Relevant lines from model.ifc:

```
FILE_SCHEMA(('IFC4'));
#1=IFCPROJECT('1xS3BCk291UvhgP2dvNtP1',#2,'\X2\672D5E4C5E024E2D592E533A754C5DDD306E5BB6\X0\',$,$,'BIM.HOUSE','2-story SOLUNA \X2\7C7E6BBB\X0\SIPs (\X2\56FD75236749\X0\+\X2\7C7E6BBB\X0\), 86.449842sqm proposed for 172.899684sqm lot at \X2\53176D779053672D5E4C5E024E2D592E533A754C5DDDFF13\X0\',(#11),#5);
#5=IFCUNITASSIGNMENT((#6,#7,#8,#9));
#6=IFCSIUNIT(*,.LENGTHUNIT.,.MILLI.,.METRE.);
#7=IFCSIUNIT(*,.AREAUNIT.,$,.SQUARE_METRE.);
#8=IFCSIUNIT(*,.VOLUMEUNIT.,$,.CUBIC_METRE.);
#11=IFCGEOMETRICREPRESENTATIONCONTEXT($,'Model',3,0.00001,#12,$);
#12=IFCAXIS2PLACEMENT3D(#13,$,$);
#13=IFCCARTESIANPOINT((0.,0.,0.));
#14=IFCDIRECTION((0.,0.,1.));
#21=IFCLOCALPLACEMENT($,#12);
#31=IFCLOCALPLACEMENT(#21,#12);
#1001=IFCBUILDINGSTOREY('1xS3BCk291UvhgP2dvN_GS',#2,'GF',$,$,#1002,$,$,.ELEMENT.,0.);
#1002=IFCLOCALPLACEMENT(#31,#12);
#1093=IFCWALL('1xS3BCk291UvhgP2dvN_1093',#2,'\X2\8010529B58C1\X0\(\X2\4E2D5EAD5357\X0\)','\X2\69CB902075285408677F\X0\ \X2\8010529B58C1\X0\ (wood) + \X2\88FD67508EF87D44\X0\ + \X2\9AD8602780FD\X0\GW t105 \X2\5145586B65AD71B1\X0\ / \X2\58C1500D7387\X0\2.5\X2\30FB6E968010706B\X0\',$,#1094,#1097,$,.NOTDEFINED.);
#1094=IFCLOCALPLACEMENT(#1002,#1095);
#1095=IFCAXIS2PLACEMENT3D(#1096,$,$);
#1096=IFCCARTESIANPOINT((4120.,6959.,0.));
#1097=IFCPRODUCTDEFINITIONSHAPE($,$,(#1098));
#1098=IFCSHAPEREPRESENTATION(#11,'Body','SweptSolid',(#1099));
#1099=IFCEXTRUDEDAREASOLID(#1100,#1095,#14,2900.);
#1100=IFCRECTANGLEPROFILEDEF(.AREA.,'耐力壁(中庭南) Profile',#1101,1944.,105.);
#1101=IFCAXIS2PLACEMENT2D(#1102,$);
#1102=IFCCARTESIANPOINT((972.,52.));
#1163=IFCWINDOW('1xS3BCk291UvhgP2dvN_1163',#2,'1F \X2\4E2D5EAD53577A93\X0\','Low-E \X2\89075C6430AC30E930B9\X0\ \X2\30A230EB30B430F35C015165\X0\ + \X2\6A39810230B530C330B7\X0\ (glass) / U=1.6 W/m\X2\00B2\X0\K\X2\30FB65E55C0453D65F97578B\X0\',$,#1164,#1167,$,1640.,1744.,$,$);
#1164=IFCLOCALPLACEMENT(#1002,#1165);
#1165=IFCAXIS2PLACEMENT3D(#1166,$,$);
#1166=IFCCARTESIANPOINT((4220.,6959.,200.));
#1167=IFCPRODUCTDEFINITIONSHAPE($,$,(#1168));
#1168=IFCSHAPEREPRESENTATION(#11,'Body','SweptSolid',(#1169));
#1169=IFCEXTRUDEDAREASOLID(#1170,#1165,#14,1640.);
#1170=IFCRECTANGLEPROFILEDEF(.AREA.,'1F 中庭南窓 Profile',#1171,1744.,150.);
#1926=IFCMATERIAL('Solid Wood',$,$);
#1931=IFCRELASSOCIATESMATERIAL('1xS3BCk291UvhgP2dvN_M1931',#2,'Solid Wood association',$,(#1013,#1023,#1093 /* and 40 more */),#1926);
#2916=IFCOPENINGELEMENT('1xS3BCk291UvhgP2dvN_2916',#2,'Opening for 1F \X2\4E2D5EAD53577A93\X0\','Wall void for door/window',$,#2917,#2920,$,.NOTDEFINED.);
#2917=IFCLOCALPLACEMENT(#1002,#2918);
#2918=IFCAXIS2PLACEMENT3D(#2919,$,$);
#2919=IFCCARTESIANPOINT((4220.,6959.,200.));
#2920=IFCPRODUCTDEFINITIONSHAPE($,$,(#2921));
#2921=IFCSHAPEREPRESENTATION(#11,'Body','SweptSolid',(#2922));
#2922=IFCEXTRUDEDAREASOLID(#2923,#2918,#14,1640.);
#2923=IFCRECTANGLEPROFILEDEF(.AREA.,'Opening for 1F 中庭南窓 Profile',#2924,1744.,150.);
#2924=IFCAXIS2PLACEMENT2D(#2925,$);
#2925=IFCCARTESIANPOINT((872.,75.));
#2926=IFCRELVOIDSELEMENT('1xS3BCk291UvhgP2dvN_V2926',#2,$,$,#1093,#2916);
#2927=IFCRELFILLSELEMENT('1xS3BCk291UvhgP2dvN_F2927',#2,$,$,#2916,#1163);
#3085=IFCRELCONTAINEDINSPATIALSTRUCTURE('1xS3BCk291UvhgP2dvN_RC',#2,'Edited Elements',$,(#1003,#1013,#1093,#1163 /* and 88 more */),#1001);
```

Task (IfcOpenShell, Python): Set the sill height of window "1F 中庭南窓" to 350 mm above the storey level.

```python
import numpy as np
import ifcopenshell
import ifcopenshell.api.geometry
import ifcopenshell.geom
import ifcopenshell.util.element
import ifcopenshell.util.placement
import ifcopenshell.util.shape
import ifcopenshell.util.unit

model = ifcopenshell.open("model.ifc")
unit_scale = ifcopenshell.util.unit.calculate_unit_scale(model)

window = model.by_guid("1xS3BCk291UvhgP2dvN_1163")
opening = window.FillsVoids[0].RelatingOpeningElement
storey = ifcopenshell.util.element.get_container(window, ifc_class="IfcBuildingStorey")
level = ifcopenshell.util.placement.get_local_placement(storey.ObjectPlacement)[2, 3]

# The opening's origin need not be at the sill, so measure its lowest point.
shape = ifcopenshell.geom.create_shape(ifcopenshell.geom.settings(), opening)
bottom = ifcopenshell.util.shape.get_shape_bottom_elevation(shape, shape.geometry) / unit_scale
dz = level + 0.35 / unit_scale - bottom

shift = np.array([0.0, 0.0, dz])
# The window is not placed relative to its opening, so move both.
for product in (opening, window):
    matrix = ifcopenshell.util.placement.get_local_placement(product.ObjectPlacement)
    matrix[:3, 3] += shift
    ifcopenshell.api.geometry.edit_object_placement(model, product=product, matrix=matrix, is_si=False)

print(f"moved by {dz * unit_scale:+.3f} m")

model.write("model_v2.ifc")
```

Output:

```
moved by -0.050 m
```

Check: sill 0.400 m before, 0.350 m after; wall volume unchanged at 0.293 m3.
